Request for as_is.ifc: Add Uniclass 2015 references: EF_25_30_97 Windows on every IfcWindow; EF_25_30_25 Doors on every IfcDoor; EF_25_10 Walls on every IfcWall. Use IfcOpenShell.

First a look at what the model holds.

```python
import ifcopenshell

model = ifcopenshell.open("as_is.ifc")
print(model.schema)
print("classifications:", [c.Name for c in model.by_type("IfcClassification")])
for ifc_class in ("IfcDoor", "IfcRoof", "IfcStair", "IfcWall", "IfcWindow"):
    print(ifc_class, len(model.by_type(ifc_class)))
```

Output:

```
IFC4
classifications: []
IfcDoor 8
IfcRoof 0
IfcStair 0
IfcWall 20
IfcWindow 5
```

```python
import ifcopenshell
import ifcopenshell.api.classification

model = ifcopenshell.open("as_is.ifc")

system = ifcopenshell.api.classification.add_classification(model, classification="Uniclass 2015")

codes = {
    "IfcWindow": ("EF_25_30_97", "Windows"),
    "IfcDoor": ("EF_25_30_25", "Doors"),
    "IfcWall": ("EF_25_10", "Walls"),
}
for ifc_class, (code, name) in codes.items():
    products = model.by_type(ifc_class)
    ifcopenshell.api.classification.add_reference(
        model, products=products, classification=system, identification=code, name=name
    )
    print(code, len(products))

model.write("as_is-out.ifc")
```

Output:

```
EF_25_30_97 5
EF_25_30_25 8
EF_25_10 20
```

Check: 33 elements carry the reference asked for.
